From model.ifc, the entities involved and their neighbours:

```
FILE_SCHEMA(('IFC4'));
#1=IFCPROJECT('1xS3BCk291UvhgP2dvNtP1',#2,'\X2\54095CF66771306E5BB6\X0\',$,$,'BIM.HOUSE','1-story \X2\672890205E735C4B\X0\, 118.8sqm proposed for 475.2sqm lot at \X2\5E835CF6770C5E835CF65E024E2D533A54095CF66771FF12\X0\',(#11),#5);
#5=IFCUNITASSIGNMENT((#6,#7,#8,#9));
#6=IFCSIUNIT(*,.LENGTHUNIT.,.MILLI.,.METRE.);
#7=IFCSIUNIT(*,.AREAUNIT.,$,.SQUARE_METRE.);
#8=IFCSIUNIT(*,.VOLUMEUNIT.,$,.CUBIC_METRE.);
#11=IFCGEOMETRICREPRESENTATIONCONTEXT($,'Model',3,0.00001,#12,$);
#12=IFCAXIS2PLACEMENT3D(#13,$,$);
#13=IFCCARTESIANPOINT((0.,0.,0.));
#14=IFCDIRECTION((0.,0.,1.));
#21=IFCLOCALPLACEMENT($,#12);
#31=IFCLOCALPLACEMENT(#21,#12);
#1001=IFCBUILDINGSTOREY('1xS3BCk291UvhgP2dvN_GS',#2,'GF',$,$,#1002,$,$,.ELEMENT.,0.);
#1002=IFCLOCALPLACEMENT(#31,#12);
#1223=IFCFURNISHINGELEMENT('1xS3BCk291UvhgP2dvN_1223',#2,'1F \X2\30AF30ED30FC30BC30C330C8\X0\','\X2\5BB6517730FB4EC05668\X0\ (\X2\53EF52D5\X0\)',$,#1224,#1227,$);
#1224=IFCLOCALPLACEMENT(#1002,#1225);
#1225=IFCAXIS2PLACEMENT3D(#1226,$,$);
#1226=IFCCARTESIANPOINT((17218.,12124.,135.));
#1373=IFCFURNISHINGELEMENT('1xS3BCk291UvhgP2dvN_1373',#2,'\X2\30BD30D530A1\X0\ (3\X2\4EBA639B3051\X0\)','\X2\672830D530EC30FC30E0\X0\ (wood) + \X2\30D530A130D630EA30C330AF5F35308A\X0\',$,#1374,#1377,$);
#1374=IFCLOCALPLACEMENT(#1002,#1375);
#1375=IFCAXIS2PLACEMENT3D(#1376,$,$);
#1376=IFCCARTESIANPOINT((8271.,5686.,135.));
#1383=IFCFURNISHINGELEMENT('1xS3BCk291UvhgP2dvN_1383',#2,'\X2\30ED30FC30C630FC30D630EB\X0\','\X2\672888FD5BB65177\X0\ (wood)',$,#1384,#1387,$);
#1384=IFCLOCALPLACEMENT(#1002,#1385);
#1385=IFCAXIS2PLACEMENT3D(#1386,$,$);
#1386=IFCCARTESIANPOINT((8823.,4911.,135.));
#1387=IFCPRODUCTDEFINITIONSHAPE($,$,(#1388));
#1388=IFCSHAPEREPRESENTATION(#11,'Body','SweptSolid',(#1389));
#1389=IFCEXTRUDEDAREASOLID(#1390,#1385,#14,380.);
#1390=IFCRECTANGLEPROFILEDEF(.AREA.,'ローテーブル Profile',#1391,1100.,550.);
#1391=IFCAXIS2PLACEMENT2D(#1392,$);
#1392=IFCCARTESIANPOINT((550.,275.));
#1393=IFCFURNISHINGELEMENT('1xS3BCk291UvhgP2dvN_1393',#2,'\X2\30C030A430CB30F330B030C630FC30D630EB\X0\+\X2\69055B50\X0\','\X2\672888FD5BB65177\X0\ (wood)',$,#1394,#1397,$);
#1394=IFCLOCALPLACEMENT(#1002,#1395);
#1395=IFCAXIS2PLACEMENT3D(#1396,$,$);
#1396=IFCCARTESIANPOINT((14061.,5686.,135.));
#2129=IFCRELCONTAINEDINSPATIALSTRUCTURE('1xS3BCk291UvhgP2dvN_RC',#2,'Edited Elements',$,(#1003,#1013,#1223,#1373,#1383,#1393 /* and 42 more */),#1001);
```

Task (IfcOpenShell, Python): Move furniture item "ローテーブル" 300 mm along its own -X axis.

```python
import ifcopenshell
import ifcopenshell.api.geometry
import ifcopenshell.util.placement
import ifcopenshell.util.unit

model = ifcopenshell.open("model.ifc")
unit_scale = ifcopenshell.util.unit.calculate_unit_scale(model)

item = model.by_guid("1xS3BCk291UvhgP2dvN_1383")
matrix = ifcopenshell.util.placement.get_local_placement(item.ObjectPlacement)
matrix[:3, 3] -= matrix[:3, 0] * 0.3 / unit_scale
ifcopenshell.api.geometry.edit_object_placement(model, product=item, matrix=matrix, is_si=False)

print(ifcopenshell.util.placement.get_local_placement(item.ObjectPlacement).round(3) + 0.0)

model.write("model_edited.ifc")
```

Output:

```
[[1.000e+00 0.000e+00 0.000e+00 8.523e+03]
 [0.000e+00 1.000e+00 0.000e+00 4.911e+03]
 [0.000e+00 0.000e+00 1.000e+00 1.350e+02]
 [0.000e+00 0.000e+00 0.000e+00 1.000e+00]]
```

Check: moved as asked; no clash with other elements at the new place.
